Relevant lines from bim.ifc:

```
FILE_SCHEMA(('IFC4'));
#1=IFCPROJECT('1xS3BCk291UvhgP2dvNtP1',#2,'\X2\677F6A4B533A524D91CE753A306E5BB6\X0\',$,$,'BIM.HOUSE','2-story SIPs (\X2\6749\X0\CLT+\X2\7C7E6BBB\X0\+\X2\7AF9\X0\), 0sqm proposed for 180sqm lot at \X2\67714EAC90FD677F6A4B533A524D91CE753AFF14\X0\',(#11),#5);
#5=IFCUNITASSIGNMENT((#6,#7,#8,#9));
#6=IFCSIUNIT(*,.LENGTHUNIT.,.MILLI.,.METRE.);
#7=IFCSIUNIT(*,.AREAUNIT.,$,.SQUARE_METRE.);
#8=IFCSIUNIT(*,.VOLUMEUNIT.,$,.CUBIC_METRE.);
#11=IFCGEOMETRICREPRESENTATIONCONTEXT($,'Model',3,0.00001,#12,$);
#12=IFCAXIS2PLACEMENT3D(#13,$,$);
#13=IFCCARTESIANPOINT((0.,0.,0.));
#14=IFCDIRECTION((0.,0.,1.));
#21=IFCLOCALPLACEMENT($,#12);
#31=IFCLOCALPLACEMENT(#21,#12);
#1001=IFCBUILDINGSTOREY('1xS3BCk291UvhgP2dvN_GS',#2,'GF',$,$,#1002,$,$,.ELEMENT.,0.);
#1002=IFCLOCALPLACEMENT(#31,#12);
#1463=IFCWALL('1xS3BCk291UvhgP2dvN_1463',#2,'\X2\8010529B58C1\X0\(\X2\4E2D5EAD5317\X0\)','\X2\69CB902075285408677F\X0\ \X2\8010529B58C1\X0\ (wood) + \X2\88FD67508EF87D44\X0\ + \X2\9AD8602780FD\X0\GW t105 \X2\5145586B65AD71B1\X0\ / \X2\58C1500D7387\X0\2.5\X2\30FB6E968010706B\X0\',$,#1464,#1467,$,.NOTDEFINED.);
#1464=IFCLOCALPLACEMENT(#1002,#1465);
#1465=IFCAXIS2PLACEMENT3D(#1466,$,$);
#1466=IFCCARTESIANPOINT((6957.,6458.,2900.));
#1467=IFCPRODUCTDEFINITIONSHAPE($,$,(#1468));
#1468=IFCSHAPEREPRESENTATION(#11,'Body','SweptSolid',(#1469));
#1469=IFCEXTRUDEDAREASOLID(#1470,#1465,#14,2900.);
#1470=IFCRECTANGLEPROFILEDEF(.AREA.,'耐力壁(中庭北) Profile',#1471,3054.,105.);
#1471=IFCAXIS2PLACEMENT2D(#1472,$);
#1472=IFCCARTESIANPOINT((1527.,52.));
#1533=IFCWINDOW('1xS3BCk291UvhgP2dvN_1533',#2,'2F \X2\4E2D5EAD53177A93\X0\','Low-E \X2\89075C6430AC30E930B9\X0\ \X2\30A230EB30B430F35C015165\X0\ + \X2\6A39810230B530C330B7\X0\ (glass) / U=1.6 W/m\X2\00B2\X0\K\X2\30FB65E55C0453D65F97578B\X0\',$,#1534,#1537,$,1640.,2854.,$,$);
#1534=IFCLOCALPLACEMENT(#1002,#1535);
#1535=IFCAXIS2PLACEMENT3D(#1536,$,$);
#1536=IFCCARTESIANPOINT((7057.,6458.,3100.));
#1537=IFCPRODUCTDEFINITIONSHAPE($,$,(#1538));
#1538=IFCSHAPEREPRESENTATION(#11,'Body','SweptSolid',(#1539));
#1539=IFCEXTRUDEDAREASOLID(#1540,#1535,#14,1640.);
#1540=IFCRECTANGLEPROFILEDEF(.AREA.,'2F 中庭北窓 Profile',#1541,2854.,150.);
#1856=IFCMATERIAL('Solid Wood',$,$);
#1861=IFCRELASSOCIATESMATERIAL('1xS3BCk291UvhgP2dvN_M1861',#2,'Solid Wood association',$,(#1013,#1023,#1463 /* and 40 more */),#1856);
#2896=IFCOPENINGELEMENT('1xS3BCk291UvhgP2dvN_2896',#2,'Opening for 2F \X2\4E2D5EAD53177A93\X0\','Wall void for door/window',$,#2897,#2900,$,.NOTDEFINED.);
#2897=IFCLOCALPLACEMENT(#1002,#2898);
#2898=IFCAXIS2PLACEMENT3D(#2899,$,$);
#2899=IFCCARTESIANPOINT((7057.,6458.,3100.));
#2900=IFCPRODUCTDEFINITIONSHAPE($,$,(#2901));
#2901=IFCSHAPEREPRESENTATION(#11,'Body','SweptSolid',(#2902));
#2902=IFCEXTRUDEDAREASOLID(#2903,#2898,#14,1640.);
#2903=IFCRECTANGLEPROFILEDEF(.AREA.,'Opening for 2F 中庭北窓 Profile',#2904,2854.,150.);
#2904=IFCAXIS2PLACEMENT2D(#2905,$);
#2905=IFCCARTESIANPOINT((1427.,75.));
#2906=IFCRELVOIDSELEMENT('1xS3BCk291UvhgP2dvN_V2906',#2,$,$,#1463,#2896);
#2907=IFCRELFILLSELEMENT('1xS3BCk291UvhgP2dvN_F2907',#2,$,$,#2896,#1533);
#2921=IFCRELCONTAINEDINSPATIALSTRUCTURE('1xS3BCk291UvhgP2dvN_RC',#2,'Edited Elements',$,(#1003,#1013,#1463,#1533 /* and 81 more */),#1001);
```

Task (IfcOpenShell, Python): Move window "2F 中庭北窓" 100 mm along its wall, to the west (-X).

```python
import ifcopenshell
import ifcopenshell.api.geometry
import ifcopenshell.util.placement
import ifcopenshell.util.unit

model = ifcopenshell.open("bim.ifc")
unit_scale = ifcopenshell.util.unit.calculate_unit_scale(model)

window = model.by_guid("1xS3BCk291UvhgP2dvN_1533")
opening = window.FillsVoids[0].RelatingOpeningElement
wall = opening.VoidsElements[0].RelatingBuildingElement

wall_matrix = ifcopenshell.util.placement.get_local_placement(wall.ObjectPlacement)
shift = wall_matrix[:3, 0] * -0.1 / unit_scale
before = ifcopenshell.util.placement.get_local_placement(window.ObjectPlacement)[:3, 3].copy()

# The window is not placed relative to its opening, so move both.
for product in (opening, window):
    matrix = ifcopenshell.util.placement.get_local_placement(product.ObjectPlacement)
    matrix[:3, 3] += shift
    ifcopenshell.api.geometry.edit_object_placement(model, product=product, matrix=matrix, is_si=False)

after = ifcopenshell.util.placement.get_local_placement(window.ObjectPlacement)[:3, 3]
print("window moved by", (after - before).round(3) + 0.0)

model.write("bim_rev.ifc")
```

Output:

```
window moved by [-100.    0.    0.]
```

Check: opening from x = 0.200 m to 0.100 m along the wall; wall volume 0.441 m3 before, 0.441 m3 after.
